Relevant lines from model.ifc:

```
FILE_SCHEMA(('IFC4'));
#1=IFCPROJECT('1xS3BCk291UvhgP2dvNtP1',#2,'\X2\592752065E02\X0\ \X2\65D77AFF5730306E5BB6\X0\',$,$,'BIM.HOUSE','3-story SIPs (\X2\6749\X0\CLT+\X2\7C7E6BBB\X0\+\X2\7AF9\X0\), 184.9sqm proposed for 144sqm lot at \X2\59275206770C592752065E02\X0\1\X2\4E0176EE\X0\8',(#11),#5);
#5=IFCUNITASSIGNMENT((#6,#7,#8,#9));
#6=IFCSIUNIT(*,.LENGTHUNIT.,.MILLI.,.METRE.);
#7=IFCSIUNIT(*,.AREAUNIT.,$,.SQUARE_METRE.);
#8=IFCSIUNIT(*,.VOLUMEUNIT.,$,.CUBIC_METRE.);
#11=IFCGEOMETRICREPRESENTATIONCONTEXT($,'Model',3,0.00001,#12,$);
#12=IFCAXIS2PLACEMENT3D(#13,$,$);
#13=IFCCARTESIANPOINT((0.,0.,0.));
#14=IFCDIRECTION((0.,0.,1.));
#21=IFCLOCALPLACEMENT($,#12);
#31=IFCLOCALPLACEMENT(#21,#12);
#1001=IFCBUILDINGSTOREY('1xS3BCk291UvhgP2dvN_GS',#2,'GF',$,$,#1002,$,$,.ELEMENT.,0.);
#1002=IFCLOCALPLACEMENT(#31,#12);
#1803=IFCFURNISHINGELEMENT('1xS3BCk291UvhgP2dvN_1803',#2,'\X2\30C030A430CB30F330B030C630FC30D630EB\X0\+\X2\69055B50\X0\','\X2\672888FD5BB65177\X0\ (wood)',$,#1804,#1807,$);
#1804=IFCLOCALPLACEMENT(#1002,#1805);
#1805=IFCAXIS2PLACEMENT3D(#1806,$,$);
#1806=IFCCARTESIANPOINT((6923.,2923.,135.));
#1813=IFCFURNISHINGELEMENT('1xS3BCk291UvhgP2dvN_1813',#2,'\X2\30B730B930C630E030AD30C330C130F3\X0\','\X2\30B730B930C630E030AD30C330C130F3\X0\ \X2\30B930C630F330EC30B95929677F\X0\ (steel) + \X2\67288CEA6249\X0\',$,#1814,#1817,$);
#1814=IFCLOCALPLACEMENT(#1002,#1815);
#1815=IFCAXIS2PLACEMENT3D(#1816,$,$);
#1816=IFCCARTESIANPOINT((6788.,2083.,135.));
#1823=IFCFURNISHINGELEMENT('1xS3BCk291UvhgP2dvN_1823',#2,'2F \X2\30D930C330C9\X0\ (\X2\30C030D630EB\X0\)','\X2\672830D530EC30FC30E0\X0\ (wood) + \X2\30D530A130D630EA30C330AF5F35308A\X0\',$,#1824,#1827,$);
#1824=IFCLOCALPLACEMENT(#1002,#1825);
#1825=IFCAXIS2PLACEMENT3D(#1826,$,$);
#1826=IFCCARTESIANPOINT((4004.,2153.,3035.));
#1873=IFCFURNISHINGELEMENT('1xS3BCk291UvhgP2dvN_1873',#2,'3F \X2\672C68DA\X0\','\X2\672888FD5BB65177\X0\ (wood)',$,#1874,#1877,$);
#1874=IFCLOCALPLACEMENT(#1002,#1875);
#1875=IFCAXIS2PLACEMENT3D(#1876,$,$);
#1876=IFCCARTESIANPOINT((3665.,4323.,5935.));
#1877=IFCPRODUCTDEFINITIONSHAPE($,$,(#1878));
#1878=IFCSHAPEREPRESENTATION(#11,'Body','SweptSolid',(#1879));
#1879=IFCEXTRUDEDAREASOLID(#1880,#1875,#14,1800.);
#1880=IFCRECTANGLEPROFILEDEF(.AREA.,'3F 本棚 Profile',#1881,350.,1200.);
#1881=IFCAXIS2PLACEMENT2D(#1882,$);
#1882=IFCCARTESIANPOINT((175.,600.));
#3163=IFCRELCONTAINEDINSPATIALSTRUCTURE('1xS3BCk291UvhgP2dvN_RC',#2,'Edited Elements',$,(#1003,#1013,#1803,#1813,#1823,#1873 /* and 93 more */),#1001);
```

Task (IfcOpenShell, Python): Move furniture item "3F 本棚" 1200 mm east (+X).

```python
import ifcopenshell
import ifcopenshell.api.geometry
import ifcopenshell.util.placement
import ifcopenshell.util.unit

model = ifcopenshell.open("model.ifc")
unit_scale = ifcopenshell.util.unit.calculate_unit_scale(model)

item = model.by_id(1873)
matrix = ifcopenshell.util.placement.get_local_placement(item.ObjectPlacement)
matrix[0, 3] += 1.2 / unit_scale
ifcopenshell.api.geometry.edit_object_placement(model, product=item, matrix=matrix, is_si=False)

print(ifcopenshell.util.placement.get_local_placement(item.ObjectPlacement).round(3) + 0.0)

model.write("model-out.ifc")
```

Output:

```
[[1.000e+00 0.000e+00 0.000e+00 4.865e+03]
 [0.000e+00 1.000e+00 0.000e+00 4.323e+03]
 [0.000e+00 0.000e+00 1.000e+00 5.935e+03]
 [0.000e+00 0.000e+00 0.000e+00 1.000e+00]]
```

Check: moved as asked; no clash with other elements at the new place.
